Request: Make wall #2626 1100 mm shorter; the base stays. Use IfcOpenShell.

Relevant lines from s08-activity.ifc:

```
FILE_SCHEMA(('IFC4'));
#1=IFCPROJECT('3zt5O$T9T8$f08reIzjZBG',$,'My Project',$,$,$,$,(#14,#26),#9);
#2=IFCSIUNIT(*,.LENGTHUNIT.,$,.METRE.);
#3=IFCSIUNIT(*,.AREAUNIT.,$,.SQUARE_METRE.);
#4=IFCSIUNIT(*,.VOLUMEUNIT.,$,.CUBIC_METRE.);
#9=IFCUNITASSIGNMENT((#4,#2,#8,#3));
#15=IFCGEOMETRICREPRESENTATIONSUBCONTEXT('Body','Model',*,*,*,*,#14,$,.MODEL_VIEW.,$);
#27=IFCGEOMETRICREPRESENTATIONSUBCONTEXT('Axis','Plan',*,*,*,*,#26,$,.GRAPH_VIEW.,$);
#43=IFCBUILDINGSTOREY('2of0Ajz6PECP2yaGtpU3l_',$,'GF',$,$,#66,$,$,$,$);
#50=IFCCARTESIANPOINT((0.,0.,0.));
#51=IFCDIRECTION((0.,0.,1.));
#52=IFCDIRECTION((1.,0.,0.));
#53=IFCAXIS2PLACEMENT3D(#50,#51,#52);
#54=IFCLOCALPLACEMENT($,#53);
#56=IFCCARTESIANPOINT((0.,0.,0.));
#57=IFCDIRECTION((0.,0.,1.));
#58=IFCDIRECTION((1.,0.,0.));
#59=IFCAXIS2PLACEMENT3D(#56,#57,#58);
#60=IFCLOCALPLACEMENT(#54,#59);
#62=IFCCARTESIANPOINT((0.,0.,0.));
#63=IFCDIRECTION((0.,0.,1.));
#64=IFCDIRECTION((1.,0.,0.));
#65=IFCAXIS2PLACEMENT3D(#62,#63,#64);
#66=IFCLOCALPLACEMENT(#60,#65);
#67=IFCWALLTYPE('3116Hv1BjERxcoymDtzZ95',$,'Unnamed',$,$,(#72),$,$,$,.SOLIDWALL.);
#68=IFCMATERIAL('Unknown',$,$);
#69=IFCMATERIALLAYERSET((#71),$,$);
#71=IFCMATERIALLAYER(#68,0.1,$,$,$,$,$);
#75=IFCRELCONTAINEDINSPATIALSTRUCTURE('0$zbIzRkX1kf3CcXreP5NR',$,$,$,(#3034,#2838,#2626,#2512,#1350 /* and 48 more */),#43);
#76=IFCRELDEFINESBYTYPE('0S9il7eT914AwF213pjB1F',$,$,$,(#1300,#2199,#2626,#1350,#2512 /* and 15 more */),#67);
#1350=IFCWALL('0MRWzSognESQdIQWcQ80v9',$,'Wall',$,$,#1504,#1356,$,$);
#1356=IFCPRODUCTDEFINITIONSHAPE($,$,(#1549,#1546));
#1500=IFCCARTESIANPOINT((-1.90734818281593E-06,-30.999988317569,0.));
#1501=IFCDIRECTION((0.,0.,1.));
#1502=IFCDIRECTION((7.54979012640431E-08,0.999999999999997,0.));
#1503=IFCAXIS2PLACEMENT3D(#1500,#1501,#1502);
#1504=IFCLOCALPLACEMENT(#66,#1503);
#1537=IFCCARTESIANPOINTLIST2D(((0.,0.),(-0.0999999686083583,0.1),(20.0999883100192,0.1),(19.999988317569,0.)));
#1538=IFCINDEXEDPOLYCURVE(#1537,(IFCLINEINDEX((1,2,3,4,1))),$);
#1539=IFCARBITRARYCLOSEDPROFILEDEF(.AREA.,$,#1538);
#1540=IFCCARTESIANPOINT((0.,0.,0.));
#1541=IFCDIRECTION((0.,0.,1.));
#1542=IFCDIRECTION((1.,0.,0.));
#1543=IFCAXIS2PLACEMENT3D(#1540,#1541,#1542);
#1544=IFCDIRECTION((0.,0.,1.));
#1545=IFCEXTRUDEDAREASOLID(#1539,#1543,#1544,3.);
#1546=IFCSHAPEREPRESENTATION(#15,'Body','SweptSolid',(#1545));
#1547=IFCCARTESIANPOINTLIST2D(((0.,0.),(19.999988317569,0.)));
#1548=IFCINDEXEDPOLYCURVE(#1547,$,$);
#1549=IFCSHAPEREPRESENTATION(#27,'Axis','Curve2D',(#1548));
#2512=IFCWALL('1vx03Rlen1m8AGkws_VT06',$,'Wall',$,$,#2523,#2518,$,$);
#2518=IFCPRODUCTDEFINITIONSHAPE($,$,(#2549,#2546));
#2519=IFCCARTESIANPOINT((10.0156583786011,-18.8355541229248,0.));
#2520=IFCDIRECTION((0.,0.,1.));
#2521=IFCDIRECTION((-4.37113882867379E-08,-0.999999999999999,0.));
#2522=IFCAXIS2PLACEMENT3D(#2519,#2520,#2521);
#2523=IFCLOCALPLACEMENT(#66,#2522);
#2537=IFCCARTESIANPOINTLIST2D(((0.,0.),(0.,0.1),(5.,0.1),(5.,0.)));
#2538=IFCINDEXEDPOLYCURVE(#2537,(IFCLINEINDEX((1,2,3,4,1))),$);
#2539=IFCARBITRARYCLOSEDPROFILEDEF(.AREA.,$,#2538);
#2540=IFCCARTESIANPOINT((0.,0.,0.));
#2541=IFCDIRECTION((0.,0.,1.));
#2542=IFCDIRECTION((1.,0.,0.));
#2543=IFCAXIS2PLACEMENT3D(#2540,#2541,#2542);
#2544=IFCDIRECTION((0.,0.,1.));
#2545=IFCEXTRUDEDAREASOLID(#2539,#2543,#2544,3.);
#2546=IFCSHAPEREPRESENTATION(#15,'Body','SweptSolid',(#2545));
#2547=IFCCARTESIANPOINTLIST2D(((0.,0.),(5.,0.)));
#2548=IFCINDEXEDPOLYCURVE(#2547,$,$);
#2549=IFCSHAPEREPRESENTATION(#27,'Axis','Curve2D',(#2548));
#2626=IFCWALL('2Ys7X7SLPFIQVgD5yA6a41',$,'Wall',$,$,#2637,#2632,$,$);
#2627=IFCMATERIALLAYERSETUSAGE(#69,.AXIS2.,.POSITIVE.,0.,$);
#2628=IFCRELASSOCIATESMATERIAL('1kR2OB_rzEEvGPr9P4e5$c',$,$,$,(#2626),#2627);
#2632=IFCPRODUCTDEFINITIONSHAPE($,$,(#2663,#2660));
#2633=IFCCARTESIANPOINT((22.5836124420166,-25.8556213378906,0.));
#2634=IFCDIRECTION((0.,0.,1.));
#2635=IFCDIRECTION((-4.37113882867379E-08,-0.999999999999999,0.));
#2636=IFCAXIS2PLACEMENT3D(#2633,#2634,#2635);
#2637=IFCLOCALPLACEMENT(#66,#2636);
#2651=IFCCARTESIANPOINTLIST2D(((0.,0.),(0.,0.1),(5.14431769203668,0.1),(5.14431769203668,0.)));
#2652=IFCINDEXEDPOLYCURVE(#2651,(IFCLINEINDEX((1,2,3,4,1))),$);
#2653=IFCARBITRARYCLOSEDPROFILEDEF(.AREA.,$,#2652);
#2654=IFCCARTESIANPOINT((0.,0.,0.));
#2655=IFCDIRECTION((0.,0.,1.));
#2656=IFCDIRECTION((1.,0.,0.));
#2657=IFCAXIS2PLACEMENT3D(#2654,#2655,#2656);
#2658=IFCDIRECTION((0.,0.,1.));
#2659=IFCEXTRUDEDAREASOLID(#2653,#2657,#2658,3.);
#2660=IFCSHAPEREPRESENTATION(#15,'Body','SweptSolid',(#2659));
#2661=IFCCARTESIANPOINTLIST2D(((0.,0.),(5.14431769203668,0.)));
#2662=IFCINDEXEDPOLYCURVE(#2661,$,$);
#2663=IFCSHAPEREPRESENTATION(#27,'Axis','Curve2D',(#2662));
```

```python
import ifcopenshell
import ifcopenshell.geom
import ifcopenshell.util.representation
import ifcopenshell.util.shape
import ifcopenshell.util.unit

model = ifcopenshell.open("s08-activity.ifc")
unit_scale = ifcopenshell.util.unit.calculate_unit_scale(model)
settings = ifcopenshell.geom.settings()


def volume(element):
    """Net volume in cubic metres, openings subtracted."""
    shape = ifcopenshell.geom.create_shape(settings, element)
    return ifcopenshell.util.shape.get_volume(shape.geometry)


wall = model.by_guid("2Ys7X7SLPFIQVgD5yA6a41")
before = volume(wall)

body = ifcopenshell.util.representation.get_representation(wall, "Model", "Body")
solid = body.Items[0]
old_height = solid.Depth
solid.Depth -= 1.1 / unit_scale
after = volume(wall)

print(f"height {old_height:g} -> {solid.Depth:g}, volume {before:.3f} -> {after:.3f} m3")

model.write("s08-activity_updated.ifc")
```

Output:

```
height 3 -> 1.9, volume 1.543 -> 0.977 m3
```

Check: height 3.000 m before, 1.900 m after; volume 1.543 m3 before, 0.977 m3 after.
